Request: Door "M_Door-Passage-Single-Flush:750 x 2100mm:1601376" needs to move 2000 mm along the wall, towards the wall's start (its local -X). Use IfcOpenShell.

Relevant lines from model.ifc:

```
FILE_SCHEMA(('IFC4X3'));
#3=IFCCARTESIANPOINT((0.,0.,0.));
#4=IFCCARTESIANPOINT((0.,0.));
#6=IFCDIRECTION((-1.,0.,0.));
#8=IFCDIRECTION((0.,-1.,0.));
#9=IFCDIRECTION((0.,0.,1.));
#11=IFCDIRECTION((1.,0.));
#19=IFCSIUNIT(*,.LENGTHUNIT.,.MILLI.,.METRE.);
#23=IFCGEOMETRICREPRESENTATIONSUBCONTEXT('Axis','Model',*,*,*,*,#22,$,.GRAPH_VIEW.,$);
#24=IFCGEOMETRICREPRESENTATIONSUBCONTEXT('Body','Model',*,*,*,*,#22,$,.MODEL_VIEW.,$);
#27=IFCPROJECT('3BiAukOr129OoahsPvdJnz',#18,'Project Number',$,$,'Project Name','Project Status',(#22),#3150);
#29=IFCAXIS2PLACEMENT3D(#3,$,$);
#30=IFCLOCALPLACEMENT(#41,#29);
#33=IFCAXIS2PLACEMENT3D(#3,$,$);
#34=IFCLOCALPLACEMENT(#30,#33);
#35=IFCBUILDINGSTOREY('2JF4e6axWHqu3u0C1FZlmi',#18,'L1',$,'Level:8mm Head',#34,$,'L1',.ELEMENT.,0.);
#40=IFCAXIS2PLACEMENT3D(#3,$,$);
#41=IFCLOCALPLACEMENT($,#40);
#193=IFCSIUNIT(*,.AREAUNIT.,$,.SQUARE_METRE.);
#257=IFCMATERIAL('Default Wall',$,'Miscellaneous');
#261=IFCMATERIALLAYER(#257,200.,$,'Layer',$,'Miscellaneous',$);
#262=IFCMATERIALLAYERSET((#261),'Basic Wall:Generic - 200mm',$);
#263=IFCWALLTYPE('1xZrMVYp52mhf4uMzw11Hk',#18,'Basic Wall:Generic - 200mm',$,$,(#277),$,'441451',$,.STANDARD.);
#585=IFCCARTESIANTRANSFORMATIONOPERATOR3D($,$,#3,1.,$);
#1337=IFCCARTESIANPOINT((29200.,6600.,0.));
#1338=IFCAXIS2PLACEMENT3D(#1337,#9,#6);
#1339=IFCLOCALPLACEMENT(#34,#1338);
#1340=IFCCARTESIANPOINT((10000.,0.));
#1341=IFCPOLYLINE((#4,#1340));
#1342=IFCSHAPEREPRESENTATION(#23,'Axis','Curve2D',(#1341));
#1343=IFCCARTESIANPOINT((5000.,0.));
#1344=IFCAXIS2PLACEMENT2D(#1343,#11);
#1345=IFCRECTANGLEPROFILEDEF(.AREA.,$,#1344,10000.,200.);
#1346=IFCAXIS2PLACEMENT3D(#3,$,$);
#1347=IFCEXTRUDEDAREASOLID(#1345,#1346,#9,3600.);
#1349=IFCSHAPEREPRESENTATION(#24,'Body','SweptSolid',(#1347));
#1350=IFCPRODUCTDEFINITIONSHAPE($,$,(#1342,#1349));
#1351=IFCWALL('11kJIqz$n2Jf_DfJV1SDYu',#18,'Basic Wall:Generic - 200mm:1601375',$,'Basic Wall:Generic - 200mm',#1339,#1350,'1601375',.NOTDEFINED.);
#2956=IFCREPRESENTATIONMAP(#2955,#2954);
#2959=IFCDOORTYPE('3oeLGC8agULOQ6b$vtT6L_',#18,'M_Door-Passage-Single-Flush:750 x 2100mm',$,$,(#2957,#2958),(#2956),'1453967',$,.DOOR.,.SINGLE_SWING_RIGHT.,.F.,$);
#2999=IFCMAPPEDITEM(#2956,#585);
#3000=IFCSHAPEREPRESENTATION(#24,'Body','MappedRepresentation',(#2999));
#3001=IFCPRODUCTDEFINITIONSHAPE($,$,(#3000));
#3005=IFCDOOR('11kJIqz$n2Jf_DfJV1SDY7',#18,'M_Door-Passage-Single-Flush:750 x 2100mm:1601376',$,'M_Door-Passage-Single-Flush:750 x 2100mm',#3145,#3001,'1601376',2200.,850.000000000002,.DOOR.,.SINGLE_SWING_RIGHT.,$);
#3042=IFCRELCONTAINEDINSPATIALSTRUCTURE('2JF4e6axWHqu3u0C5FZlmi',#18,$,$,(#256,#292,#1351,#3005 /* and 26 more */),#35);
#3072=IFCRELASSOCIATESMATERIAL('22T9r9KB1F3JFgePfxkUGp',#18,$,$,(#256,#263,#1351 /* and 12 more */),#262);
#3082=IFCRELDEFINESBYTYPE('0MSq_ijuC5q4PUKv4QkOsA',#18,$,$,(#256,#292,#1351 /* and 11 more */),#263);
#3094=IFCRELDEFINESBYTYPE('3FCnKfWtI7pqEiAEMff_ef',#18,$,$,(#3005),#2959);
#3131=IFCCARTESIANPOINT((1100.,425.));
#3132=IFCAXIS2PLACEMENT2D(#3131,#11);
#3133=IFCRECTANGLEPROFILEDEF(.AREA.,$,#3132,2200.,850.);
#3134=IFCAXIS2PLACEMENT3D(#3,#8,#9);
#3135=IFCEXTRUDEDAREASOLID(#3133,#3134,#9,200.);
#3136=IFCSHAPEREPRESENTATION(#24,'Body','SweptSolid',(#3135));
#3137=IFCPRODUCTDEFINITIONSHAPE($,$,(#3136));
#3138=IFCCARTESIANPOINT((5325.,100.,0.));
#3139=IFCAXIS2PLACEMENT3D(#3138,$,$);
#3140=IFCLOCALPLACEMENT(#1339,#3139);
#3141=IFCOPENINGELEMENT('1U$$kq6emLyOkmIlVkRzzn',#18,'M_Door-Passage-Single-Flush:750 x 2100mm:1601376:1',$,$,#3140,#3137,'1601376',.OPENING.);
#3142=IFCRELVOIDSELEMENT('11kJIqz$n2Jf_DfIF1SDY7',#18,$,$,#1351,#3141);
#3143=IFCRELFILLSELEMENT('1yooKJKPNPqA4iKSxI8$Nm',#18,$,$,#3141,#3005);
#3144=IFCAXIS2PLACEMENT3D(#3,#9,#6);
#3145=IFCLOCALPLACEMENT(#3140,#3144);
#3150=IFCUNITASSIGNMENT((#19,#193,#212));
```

```python
import ifcopenshell
import ifcopenshell.api.geometry
import ifcopenshell.util.placement
import ifcopenshell.util.unit

model = ifcopenshell.open("model.ifc")
unit_scale = ifcopenshell.util.unit.calculate_unit_scale(model)

door = model.by_guid("11kJIqz$n2Jf_DfJV1SDY7")
opening = door.FillsVoids[0].RelatingOpeningElement
wall = opening.VoidsElements[0].RelatingBuildingElement

wall_matrix = ifcopenshell.util.placement.get_local_placement(wall.ObjectPlacement)
shift = wall_matrix[:3, 0] * -2 / unit_scale
before = ifcopenshell.util.placement.get_local_placement(door.ObjectPlacement)[:3, 3].copy()

# The door is placed relative to its opening, so it follows when the opening moves.
matrix = ifcopenshell.util.placement.get_local_placement(opening.ObjectPlacement)
matrix[:3, 3] += shift
ifcopenshell.api.geometry.edit_object_placement(
    model, product=opening, matrix=matrix, is_si=False, should_transform_children=True
)

after = ifcopenshell.util.placement.get_local_placement(door.ObjectPlacement)[:3, 3]
print("door moved by", (after - before).round(3) + 0.0)

model.write("model_edited.ifc")
```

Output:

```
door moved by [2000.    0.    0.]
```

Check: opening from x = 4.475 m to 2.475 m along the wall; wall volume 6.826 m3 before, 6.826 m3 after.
